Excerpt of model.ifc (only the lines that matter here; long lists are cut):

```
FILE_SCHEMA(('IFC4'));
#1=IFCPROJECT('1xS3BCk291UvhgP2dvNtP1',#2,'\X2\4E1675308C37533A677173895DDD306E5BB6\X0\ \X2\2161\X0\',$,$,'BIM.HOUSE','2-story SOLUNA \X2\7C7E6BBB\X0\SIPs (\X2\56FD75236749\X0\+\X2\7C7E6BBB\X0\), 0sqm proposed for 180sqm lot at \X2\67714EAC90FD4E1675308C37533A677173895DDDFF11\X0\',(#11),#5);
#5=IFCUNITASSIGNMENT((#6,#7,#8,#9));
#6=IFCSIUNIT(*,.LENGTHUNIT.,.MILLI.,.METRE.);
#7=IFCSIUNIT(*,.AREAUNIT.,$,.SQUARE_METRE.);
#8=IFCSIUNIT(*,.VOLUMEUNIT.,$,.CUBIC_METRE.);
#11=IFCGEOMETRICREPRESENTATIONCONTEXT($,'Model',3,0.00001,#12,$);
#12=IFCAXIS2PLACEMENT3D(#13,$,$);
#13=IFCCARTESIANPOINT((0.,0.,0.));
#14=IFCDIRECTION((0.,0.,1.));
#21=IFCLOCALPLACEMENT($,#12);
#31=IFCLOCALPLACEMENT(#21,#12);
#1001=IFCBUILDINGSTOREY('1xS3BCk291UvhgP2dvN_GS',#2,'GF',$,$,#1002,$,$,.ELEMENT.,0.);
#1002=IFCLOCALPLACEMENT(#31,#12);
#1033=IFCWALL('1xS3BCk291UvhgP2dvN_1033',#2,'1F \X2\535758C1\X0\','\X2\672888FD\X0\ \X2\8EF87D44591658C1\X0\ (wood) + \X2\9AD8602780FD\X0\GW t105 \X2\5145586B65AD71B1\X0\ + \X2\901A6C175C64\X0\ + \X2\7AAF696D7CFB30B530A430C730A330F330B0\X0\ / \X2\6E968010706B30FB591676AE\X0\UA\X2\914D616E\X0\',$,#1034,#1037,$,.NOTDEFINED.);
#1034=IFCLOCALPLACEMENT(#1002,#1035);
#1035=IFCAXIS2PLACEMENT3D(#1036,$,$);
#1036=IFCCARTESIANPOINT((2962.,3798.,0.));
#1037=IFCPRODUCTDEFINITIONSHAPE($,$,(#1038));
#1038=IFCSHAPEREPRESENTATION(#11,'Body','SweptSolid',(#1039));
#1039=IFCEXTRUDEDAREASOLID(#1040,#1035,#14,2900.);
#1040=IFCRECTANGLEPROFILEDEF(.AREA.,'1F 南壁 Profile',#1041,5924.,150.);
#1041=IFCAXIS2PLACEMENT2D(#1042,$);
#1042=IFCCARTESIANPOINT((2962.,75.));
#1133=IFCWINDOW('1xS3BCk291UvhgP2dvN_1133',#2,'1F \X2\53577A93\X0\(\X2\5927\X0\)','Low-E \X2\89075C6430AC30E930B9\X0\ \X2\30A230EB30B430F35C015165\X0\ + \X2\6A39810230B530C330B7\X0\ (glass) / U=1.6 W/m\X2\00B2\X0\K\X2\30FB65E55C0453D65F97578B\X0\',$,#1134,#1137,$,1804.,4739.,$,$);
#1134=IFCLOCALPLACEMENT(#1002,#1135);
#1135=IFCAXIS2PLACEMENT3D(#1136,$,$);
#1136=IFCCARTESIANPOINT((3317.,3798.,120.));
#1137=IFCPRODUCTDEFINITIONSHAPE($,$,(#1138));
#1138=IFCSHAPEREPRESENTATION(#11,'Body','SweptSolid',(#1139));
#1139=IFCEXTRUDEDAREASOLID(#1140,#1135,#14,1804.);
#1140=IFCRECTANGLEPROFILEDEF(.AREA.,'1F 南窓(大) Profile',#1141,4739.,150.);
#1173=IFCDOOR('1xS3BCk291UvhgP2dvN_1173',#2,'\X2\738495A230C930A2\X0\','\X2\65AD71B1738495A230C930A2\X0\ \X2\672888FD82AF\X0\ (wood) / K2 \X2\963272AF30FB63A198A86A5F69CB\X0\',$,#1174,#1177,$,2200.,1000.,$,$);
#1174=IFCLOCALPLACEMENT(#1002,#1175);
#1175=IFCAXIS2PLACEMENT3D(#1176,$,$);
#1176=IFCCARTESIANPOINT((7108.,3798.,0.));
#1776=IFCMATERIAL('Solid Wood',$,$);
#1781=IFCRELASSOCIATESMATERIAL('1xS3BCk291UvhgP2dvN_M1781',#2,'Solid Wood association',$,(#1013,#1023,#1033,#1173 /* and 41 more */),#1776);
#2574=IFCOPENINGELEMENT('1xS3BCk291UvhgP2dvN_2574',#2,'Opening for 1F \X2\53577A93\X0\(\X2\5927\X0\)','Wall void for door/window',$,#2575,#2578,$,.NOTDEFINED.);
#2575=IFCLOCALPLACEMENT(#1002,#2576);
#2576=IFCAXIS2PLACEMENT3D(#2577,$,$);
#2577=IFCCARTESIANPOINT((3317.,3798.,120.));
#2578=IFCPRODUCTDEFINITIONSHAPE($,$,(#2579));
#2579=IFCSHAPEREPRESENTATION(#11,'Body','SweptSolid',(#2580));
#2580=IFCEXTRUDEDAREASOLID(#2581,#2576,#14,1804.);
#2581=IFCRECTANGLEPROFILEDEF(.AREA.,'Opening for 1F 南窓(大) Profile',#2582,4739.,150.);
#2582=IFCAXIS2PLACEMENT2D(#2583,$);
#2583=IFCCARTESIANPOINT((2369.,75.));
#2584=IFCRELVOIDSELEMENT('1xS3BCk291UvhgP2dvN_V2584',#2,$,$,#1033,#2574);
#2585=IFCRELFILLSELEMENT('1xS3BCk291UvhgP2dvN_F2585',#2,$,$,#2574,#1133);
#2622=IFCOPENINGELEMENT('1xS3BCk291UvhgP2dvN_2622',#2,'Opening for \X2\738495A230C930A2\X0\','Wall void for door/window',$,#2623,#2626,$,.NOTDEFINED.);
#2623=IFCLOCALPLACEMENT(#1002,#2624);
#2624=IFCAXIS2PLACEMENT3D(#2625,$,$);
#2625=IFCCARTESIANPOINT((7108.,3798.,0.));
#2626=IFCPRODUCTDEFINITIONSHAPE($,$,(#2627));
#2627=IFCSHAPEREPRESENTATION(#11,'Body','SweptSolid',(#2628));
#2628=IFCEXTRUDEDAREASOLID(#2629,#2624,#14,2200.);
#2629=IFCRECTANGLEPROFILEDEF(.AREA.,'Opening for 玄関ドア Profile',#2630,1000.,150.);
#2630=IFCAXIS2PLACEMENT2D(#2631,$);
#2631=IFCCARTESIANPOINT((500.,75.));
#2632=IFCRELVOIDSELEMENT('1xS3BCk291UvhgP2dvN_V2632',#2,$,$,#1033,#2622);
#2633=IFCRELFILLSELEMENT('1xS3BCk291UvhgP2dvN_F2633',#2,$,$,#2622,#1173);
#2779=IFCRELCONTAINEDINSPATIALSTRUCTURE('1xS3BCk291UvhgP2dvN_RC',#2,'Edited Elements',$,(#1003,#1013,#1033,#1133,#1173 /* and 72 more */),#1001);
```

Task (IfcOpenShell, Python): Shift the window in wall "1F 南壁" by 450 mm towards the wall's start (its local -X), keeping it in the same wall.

```python
import ifcopenshell
import ifcopenshell.api.geometry
import ifcopenshell.util.placement
import ifcopenshell.util.unit

model = ifcopenshell.open("model.ifc")
unit_scale = ifcopenshell.util.unit.calculate_unit_scale(model)

window = model.by_id(1133)
opening = window.FillsVoids[0].RelatingOpeningElement
wall = opening.VoidsElements[0].RelatingBuildingElement

wall_matrix = ifcopenshell.util.placement.get_local_placement(wall.ObjectPlacement)
shift = wall_matrix[:3, 0] * -0.45 / unit_scale
before = ifcopenshell.util.placement.get_local_placement(window.ObjectPlacement)[:3, 3].copy()

# The window is not placed relative to its opening, so move both.
for product in (opening, window):
    matrix = ifcopenshell.util.placement.get_local_placement(product.ObjectPlacement)
    matrix[:3, 3] += shift
    ifcopenshell.api.geometry.edit_object_placement(model, product=product, matrix=matrix, is_si=False)

after = ifcopenshell.util.placement.get_local_placement(window.ObjectPlacement)[:3, 3]
print("window moved by", (after - before).round(3) + 0.0)

model.write("model_edited.ifc")
```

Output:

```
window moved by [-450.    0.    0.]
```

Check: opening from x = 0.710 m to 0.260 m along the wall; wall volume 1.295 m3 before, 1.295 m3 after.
